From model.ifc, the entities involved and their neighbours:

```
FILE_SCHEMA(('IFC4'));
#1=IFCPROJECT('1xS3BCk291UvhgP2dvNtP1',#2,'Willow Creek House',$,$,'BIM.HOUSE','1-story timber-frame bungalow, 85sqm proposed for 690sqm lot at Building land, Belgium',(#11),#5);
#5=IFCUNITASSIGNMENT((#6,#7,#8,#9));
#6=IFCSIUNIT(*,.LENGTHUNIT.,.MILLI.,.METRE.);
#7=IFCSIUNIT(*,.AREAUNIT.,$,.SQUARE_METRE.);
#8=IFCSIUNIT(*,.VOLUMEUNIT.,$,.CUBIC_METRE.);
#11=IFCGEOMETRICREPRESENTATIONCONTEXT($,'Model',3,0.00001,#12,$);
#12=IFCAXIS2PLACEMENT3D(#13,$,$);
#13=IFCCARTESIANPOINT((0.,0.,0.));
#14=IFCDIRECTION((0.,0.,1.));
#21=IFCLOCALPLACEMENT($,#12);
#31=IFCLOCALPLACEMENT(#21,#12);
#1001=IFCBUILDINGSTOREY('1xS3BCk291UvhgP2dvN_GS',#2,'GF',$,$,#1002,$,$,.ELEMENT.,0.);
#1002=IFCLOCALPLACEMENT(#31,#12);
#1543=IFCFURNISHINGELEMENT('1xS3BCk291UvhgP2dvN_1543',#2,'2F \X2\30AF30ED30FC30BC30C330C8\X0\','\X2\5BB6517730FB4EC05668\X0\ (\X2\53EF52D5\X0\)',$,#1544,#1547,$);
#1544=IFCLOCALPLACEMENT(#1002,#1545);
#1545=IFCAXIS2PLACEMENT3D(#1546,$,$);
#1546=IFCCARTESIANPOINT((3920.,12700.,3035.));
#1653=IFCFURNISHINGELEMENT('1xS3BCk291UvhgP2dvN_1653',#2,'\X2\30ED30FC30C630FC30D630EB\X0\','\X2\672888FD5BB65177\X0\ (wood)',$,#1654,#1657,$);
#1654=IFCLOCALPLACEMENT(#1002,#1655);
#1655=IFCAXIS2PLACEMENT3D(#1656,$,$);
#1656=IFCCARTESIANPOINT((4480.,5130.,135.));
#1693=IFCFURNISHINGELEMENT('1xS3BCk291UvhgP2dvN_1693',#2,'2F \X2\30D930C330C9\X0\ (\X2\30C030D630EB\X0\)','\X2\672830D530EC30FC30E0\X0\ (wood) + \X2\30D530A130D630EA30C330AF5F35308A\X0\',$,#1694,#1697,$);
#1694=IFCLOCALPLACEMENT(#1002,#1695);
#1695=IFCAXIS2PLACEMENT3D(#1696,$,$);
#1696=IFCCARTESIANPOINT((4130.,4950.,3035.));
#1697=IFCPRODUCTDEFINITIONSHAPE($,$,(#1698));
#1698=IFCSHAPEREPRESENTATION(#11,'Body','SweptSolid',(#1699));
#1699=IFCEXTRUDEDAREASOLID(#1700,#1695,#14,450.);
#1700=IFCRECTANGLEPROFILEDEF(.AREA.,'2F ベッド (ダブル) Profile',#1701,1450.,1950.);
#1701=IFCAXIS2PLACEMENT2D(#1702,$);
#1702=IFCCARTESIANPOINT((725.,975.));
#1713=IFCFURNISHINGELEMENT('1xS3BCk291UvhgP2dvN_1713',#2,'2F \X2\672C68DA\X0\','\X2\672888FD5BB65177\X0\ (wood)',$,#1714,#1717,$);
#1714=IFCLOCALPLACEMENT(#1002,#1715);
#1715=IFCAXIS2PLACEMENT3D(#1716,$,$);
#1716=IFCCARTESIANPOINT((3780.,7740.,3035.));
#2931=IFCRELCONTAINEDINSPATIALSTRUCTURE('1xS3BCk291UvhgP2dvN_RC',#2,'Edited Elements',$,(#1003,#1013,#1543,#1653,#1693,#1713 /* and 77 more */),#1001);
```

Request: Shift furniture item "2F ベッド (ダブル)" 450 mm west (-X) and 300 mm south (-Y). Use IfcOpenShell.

```python
import ifcopenshell
import ifcopenshell.api.geometry
import ifcopenshell.util.placement

model = ifcopenshell.open("model.ifc")

item = model.by_guid("1xS3BCk291UvhgP2dvN_1693")
matrix = ifcopenshell.util.placement.get_local_placement(item.ObjectPlacement)
matrix[0, 3] -= 450.0
matrix[1, 3] -= 300.0
ifcopenshell.api.geometry.edit_object_placement(model, product=item, matrix=matrix, is_si=False)

print(ifcopenshell.util.placement.get_local_placement(item.ObjectPlacement).round(3) + 0.0)

model.write("model_edited.ifc")
```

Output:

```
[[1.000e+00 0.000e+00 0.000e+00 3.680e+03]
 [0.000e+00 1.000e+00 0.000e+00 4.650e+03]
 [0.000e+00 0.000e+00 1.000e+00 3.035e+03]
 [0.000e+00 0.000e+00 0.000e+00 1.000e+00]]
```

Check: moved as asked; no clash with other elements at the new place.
